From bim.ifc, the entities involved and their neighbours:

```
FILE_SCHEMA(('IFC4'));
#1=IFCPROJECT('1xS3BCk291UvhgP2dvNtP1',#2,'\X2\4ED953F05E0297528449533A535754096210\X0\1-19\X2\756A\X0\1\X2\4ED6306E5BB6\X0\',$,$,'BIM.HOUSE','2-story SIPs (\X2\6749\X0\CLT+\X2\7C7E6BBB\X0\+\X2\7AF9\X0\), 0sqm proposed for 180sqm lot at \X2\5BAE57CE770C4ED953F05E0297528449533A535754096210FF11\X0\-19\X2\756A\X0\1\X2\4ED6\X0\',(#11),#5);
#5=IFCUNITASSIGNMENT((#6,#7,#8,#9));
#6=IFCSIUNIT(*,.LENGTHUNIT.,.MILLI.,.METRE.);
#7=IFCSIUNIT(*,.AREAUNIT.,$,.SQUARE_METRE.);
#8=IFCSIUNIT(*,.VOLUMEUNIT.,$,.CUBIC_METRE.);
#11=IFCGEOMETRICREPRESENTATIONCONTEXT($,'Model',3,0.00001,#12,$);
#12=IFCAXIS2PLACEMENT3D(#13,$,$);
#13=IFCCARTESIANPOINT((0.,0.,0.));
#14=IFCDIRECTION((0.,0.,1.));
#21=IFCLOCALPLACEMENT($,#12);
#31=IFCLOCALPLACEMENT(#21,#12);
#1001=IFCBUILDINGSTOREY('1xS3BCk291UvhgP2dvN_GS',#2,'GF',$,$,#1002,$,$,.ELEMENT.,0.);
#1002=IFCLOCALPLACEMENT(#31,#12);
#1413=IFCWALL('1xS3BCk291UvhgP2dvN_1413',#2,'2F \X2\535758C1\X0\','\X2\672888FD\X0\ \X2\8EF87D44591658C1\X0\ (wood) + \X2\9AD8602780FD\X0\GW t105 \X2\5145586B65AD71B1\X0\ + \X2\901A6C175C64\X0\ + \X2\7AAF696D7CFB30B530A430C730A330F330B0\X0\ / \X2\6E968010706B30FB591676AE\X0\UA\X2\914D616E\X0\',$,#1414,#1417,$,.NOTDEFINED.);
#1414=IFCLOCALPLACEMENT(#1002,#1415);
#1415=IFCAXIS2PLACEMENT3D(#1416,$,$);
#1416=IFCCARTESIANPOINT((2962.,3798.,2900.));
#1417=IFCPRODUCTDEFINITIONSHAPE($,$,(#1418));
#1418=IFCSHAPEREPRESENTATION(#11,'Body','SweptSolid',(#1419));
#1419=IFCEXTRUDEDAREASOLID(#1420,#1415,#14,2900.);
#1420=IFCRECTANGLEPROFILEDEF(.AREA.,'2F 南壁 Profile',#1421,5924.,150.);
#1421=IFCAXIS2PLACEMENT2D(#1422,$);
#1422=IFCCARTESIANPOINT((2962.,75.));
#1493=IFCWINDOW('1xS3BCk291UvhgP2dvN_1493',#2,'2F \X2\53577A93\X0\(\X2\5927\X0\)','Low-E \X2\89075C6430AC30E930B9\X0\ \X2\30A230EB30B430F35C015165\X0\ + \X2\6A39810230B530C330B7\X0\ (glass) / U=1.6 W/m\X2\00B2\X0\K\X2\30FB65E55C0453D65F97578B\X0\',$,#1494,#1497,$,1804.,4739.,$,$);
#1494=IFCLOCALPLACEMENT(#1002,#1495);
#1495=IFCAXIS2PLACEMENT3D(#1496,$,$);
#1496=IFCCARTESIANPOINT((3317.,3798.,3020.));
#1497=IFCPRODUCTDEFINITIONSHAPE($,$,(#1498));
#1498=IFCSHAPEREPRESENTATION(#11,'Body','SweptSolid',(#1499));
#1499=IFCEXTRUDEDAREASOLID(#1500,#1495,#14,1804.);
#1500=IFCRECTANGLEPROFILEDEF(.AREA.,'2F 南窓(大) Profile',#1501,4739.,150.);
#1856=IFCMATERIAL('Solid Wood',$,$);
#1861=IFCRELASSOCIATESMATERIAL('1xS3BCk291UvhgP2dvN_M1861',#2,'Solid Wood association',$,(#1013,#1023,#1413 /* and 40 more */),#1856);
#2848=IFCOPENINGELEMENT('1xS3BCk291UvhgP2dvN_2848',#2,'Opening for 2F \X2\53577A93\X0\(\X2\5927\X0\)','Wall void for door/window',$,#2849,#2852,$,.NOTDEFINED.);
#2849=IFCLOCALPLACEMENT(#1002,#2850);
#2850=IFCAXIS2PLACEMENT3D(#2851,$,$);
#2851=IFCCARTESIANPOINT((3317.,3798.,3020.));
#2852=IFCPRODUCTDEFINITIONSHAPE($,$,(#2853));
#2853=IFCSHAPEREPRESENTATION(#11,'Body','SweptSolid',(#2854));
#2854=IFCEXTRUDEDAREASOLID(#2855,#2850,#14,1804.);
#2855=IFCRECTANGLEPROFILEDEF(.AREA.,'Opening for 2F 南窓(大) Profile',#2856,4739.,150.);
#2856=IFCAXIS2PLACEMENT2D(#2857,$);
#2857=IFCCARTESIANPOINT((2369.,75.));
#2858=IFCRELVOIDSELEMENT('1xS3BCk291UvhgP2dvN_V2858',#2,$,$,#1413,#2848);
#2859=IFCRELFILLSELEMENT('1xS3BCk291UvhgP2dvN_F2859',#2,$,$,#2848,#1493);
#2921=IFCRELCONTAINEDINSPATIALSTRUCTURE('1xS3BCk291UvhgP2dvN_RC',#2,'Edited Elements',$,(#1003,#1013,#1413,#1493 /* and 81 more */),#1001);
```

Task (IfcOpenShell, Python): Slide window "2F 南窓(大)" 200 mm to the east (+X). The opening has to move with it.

```python
import ifcopenshell
import ifcopenshell.api.geometry
import ifcopenshell.util.placement
import ifcopenshell.util.unit

model = ifcopenshell.open("bim.ifc")
unit_scale = ifcopenshell.util.unit.calculate_unit_scale(model)

window = model.by_guid("1xS3BCk291UvhgP2dvN_1493")
opening = window.FillsVoids[0].RelatingOpeningElement
wall = opening.VoidsElements[0].RelatingBuildingElement

wall_matrix = ifcopenshell.util.placement.get_local_placement(wall.ObjectPlacement)
shift = wall_matrix[:3, 0] * 0.2 / unit_scale
before = ifcopenshell.util.placement.get_local_placement(window.ObjectPlacement)[:3, 3].copy()

# The window is not placed relative to its opening, so move both.
for product in (opening, window):
    matrix = ifcopenshell.util.placement.get_local_placement(product.ObjectPlacement)
    matrix[:3, 3] += shift
    ifcopenshell.api.geometry.edit_object_placement(model, product=product, matrix=matrix, is_si=False)

after = ifcopenshell.util.placement.get_local_placement(window.ObjectPlacement)[:3, 3]
print("window moved by", (after - before).round(3) + 0.0)

model.write("bim_edited.ifc")
```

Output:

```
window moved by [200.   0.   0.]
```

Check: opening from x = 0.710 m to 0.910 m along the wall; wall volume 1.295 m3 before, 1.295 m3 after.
